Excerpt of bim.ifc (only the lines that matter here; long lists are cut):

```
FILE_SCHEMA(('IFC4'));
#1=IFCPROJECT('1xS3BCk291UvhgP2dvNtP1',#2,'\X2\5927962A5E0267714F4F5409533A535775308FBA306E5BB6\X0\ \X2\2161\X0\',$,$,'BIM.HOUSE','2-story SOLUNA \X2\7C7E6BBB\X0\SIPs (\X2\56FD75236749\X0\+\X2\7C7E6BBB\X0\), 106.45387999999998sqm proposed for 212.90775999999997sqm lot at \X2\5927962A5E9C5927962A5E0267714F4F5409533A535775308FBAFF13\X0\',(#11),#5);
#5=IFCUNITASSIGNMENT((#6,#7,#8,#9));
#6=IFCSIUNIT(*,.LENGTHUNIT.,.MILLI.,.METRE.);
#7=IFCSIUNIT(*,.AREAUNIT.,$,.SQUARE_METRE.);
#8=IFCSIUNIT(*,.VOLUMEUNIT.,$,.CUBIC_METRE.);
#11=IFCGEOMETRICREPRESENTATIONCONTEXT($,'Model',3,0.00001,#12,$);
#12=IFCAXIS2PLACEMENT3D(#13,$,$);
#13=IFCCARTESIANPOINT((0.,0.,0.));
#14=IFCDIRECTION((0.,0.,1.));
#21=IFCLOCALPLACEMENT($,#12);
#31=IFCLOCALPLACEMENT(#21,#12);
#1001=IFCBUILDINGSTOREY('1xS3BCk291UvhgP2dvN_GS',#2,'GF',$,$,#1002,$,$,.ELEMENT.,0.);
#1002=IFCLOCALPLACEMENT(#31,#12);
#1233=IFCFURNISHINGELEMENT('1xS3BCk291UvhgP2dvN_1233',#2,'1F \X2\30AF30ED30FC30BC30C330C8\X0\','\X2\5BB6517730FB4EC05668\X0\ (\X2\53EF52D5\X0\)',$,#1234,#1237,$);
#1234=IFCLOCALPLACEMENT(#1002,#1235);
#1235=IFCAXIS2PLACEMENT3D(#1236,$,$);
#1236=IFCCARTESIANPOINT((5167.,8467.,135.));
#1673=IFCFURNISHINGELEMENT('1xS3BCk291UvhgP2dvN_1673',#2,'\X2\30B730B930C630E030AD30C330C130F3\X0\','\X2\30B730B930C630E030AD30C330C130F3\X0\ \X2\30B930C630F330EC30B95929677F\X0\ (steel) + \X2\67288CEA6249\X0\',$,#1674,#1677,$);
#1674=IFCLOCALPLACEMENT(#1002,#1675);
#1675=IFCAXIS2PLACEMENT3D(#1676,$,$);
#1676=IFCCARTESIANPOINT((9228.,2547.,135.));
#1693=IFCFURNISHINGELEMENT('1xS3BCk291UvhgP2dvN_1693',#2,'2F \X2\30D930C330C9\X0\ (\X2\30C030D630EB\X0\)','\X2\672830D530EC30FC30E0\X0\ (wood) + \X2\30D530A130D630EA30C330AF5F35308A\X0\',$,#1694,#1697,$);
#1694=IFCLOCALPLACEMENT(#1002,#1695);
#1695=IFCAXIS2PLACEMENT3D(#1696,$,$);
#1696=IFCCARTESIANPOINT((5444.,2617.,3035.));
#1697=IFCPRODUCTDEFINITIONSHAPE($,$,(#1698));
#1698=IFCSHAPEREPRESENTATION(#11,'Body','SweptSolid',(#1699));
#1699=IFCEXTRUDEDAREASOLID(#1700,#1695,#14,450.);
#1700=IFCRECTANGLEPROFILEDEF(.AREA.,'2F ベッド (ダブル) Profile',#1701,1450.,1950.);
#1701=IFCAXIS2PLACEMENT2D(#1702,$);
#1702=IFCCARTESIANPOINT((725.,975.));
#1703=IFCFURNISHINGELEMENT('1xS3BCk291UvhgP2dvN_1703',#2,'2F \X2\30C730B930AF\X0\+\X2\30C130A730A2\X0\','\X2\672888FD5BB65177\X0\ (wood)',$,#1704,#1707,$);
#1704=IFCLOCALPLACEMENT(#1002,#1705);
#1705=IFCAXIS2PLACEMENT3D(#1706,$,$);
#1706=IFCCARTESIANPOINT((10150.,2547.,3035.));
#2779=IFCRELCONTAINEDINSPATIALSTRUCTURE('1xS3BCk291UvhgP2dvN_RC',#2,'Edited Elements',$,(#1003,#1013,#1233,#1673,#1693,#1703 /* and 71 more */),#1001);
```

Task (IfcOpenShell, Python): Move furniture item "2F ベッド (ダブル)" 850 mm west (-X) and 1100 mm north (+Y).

```python
import ifcopenshell
import ifcopenshell.api.geometry
import ifcopenshell.util.placement

model = ifcopenshell.open("bim.ifc")

item = model.by_guid("1xS3BCk291UvhgP2dvN_1693")
matrix = ifcopenshell.util.placement.get_local_placement(item.ObjectPlacement)
matrix[0, 3] -= 850.0
matrix[1, 3] += 1100.0
ifcopenshell.api.geometry.edit_object_placement(model, product=item, matrix=matrix, is_si=False)

print(ifcopenshell.util.placement.get_local_placement(item.ObjectPlacement).round(3) + 0.0)

model.write("bim_rev.ifc")
```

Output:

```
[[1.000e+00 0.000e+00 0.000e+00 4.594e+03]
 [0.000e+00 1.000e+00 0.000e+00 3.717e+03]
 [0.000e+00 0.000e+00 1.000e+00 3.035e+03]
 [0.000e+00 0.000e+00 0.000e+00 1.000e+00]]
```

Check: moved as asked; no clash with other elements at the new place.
